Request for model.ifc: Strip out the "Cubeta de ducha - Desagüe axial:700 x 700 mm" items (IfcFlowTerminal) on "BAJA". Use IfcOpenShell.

First a look at what the model holds.

```python
import ifcopenshell
import ifcopenshell.util.element

model = ifcopenshell.open("model.ifc")
print(model.schema)
storey = next(s for s in model.by_type("IfcBuildingStorey") if s.Name == "BAJA")
terminals = [e for e in ifcopenshell.util.element.get_decomposition(storey) if e.is_a("IfcFlowTerminal")]
seen = {}
for e in terminals:
    element_type = ifcopenshell.util.element.get_type(e)
    name = element_type.Name if element_type not in (None, e) else None
    seen[name] = seen.get(name, 0) + 1
for name, count in sorted(seen.items(), key=str):
    print(count, "x", name)
```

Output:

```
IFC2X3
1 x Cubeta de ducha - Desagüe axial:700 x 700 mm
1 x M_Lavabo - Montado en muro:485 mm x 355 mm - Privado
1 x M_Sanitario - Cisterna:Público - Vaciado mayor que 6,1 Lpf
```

```python
import ifcopenshell
import ifcopenshell.api.root
import ifcopenshell.util.element

model = ifcopenshell.open("model.ifc")

storey = next(s for s in model.by_type("IfcBuildingStorey") if s.Name == "BAJA")
terminals = [e for e in ifcopenshell.util.element.get_decomposition(storey) if e.is_a("IfcFlowTerminal")]
targets = [e for e in terminals if (t := ifcopenshell.util.element.get_type(e)) not in (None, e) and t.Name == "Cubeta de ducha - Desagüe axial:700 x 700 mm"]

for e in targets:
    ifcopenshell.api.root.remove_product(model, product=e)
print(len(targets), "removed")

model.write("model-out.ifc")
```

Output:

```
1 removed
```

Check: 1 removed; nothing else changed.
